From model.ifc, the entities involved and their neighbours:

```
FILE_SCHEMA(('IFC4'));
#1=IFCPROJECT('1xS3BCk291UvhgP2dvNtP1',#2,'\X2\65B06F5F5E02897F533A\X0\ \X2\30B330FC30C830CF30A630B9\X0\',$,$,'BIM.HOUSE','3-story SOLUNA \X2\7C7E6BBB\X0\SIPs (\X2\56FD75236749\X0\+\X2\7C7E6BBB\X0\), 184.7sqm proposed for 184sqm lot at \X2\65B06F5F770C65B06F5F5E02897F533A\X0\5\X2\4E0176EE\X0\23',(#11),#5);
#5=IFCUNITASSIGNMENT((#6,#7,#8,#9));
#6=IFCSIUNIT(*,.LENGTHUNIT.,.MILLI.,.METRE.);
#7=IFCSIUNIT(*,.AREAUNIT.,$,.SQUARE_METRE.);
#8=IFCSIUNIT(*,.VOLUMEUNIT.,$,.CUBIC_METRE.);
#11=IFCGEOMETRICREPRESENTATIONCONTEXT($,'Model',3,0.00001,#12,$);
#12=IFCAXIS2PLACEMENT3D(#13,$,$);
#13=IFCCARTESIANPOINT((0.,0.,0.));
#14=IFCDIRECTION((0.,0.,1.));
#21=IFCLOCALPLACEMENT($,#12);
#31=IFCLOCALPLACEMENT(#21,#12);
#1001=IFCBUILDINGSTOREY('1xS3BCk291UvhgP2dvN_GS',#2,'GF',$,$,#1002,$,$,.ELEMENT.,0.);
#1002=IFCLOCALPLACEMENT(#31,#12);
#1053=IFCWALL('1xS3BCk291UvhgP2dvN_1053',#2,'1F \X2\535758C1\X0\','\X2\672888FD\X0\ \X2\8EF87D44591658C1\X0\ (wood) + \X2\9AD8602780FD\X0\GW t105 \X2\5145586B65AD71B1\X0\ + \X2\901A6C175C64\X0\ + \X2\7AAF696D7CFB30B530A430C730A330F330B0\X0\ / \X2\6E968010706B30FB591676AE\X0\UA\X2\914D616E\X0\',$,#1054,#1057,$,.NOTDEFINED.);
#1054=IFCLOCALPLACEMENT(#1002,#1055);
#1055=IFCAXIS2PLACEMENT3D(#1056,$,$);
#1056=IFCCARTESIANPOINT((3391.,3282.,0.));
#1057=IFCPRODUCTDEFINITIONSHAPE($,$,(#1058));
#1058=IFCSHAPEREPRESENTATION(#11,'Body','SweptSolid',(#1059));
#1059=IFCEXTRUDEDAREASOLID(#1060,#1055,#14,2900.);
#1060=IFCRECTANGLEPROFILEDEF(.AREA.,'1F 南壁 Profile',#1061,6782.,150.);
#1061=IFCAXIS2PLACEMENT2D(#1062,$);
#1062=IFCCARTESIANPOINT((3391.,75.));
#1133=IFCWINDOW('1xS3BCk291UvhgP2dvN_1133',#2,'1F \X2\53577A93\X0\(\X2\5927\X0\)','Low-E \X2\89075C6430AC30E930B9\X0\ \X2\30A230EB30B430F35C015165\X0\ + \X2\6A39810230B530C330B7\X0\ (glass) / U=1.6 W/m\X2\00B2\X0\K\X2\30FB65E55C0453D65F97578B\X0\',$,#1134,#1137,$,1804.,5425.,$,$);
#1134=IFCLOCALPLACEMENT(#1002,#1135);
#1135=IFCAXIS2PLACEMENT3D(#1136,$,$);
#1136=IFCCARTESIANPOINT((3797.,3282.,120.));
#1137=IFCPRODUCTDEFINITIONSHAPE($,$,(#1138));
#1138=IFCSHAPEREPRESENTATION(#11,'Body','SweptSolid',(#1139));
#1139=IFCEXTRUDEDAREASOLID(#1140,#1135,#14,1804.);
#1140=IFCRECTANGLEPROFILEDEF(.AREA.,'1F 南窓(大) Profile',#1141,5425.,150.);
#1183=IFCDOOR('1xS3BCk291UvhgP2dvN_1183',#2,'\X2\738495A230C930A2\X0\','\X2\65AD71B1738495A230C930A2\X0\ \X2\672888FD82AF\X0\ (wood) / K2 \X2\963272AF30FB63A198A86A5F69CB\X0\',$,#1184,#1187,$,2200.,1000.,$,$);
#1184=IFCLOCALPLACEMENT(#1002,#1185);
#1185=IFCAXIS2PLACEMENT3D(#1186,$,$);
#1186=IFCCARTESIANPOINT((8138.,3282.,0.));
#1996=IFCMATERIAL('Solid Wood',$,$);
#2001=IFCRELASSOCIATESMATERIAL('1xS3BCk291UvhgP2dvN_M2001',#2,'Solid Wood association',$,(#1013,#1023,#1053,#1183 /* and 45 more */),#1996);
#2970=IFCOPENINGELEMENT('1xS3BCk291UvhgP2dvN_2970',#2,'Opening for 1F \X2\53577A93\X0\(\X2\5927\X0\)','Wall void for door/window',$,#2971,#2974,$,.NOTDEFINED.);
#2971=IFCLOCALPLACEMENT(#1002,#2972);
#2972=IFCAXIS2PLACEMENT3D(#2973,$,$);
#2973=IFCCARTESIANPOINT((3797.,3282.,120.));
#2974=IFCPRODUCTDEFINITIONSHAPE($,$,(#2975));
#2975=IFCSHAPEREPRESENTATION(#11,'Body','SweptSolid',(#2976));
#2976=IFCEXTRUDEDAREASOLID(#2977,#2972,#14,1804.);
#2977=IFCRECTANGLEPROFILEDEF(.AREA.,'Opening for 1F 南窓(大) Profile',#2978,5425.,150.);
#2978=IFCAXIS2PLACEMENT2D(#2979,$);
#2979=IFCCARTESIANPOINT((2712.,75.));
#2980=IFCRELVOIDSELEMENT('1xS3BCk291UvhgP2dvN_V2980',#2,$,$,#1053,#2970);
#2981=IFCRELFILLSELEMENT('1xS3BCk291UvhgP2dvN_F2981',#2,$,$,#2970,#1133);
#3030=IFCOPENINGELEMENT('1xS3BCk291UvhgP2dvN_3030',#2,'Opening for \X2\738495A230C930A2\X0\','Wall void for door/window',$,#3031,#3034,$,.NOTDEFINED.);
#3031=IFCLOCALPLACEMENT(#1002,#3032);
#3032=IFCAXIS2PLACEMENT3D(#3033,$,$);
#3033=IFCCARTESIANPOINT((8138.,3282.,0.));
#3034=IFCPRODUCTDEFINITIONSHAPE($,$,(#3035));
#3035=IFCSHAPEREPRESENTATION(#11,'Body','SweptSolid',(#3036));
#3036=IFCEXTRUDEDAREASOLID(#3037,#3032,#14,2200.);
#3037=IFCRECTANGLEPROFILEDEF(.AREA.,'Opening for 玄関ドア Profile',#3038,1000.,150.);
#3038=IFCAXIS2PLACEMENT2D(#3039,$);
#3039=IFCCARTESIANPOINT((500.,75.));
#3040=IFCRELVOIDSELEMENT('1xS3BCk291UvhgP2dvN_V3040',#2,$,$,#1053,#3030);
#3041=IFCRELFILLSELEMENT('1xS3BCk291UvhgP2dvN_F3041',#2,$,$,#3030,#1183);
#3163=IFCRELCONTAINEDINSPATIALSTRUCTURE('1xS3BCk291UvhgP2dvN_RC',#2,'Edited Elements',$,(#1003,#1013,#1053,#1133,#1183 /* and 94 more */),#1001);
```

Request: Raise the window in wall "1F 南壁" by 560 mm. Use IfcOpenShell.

```python
import numpy as np
import ifcopenshell
import ifcopenshell.api.geometry
import ifcopenshell.util.placement
import ifcopenshell.util.unit

model = ifcopenshell.open("model.ifc")
unit_scale = ifcopenshell.util.unit.calculate_unit_scale(model)

window = model.by_guid("1xS3BCk291UvhgP2dvN_1133")
opening = window.FillsVoids[0].RelatingOpeningElement
dz = 0.56 / unit_scale

shift = np.array([0.0, 0.0, dz])
# The window is not placed relative to its opening, so move both.
for product in (opening, window):
    matrix = ifcopenshell.util.placement.get_local_placement(product.ObjectPlacement)
    matrix[:3, 3] += shift
    ifcopenshell.api.geometry.edit_object_placement(model, product=product, matrix=matrix, is_si=False)

print(f"moved by {dz * unit_scale:+.3f} m")

model.write("model_rev.ifc")
```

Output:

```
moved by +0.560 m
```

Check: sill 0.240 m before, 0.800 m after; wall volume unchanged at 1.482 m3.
